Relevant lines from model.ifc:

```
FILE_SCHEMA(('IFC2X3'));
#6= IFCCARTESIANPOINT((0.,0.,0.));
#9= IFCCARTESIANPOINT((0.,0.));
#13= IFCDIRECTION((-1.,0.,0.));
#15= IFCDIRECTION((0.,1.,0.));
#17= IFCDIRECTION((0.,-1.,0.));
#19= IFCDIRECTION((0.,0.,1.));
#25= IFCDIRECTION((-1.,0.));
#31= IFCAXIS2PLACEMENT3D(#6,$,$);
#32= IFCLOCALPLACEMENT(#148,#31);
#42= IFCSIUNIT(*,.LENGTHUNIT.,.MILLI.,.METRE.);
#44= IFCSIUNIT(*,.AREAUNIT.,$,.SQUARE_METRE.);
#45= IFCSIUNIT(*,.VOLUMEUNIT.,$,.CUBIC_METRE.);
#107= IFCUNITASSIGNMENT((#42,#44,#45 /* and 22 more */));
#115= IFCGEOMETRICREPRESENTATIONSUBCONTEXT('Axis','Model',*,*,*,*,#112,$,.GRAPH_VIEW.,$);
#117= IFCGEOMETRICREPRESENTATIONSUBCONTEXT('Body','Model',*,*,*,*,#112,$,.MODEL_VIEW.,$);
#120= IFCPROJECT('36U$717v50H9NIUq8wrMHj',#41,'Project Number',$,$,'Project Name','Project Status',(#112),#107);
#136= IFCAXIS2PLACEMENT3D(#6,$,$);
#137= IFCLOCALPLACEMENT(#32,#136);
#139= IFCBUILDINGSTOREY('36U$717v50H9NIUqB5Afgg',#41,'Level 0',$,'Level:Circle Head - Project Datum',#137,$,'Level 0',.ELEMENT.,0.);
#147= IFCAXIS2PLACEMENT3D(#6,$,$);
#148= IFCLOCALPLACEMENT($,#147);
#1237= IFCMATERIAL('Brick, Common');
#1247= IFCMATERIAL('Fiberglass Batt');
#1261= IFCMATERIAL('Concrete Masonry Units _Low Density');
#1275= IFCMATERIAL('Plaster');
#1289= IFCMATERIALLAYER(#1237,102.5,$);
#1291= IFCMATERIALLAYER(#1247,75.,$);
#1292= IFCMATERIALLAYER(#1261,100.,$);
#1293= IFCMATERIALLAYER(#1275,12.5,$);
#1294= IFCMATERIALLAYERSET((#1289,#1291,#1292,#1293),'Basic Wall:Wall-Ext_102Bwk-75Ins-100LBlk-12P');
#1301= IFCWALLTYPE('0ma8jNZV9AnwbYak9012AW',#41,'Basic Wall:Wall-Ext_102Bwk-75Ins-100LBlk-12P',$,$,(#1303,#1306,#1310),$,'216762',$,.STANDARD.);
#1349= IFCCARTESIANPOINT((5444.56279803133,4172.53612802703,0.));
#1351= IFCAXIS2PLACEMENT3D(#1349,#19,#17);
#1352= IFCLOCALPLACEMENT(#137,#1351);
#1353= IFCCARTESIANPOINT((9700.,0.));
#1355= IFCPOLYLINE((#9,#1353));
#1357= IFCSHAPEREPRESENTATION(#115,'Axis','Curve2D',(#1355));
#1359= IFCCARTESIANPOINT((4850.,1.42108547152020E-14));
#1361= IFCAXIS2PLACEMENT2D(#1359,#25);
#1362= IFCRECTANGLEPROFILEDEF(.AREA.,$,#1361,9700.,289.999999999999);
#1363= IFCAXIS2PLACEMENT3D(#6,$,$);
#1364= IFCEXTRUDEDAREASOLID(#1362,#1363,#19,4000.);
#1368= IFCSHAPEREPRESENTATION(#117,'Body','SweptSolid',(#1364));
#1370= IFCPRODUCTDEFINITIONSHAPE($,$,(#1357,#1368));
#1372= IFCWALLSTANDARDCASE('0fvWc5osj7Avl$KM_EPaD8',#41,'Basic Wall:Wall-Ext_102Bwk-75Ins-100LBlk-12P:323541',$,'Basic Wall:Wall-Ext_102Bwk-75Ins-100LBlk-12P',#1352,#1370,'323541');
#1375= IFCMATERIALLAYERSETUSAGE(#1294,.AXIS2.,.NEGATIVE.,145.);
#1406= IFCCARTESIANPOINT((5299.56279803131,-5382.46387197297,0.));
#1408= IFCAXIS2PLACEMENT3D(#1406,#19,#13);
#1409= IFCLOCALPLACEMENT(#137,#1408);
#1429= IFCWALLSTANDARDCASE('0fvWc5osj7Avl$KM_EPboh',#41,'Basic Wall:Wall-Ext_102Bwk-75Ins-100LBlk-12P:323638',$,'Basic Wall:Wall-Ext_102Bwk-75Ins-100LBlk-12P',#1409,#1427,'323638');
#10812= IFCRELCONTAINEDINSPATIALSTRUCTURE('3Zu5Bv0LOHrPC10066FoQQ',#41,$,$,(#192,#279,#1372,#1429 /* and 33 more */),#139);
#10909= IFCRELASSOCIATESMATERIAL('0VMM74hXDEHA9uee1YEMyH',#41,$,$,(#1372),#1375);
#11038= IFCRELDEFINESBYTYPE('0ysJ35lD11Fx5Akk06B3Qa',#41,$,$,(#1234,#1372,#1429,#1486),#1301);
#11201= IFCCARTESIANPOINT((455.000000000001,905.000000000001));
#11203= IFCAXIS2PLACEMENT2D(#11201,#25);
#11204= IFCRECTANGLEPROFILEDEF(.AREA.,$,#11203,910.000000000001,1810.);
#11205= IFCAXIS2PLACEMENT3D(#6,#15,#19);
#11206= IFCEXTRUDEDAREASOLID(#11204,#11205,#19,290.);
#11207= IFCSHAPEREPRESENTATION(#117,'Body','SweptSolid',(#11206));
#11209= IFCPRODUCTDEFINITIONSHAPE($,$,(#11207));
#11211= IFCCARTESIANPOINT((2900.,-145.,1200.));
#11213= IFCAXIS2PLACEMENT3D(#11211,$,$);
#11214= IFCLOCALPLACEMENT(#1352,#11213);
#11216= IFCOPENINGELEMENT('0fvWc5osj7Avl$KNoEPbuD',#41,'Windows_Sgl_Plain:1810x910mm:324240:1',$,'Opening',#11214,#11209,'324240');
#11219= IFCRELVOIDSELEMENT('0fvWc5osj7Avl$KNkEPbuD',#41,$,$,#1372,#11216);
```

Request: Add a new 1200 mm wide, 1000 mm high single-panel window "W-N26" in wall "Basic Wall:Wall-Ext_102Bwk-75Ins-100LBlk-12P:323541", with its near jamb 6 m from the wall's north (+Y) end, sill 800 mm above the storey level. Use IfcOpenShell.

```python
import numpy as np
import ifcopenshell
import ifcopenshell.api.feature
import ifcopenshell.api.geometry
import ifcopenshell.api.root
import ifcopenshell.api.spatial
import ifcopenshell.api.type
import ifcopenshell.geom
import ifcopenshell.util.element
import ifcopenshell.util.placement
import ifcopenshell.util.representation
import ifcopenshell.util.shape
import ifcopenshell.util.unit

model = ifcopenshell.open("model.ifc")
unit_scale = ifcopenshell.util.unit.calculate_unit_scale(model)
settings = ifcopenshell.geom.settings()


def volume(element):
    """Net volume in cubic metres, openings subtracted."""
    shape = ifcopenshell.geom.create_shape(settings, element)
    return ifcopenshell.util.shape.get_volume(shape.geometry)


wall = model.by_guid("0fvWc5osj7Avl$KM_EPaD8")
storey = ifcopenshell.util.element.get_container(wall, ifc_class="IfcBuildingStorey")
context = ifcopenshell.util.representation.get_context(model, "Model", "Body", "MODEL_VIEW")
before = volume(wall)

width, height, from_end, sill = 1.2, 1, 6, 0.8  # metres

# The wall runs along its own X axis, and the end named is its -X end.
wall_shape = ifcopenshell.geom.create_shape(settings, wall)
x, y, z = ifcopenshell.util.shape.get_vertices(wall_shape.geometry).T
start = x.min() + from_end
face, thickness = float(y.min()), float(y.max() - y.min())
wall_matrix = ifcopenshell.util.placement.get_local_placement(wall.ObjectPlacement)
level = ifcopenshell.util.placement.get_local_placement(storey.ObjectPlacement)[2, 3]


def in_wall(x, y):
    """Placement at x, y metres in the wall's axes, at sill height."""
    matrix = wall_matrix.copy()
    matrix[:, 3] = wall_matrix @ np.array([x / unit_scale, y / unit_scale, 0.0, 1.0])
    matrix[2, 3] = level + sill / unit_scale
    return matrix


# Opening: a box that overshoots both wall faces by 50 mm.
opening = ifcopenshell.api.root.create_entity(model, ifc_class="IfcOpeningElement")
box = ifcopenshell.api.geometry.add_wall_representation(
    model, context=context, length=width, height=height, thickness=thickness + 0.1
)
ifcopenshell.api.geometry.assign_representation(model, product=opening, representation=box)
ifcopenshell.api.geometry.edit_object_placement(model, product=opening, matrix=in_wall(start, face - 0.05), is_si=False)
ifcopenshell.api.feature.add_feature(model, feature=opening, element=wall)

window = ifcopenshell.api.root.create_entity(model, ifc_class="IfcWindow", name="W-N26")
window.OverallWidth, window.OverallHeight = width / unit_scale, height / unit_scale
body = ifcopenshell.api.geometry.add_window_representation(
    model,
    context=context,
    overall_width=window.OverallWidth,
    overall_height=window.OverallHeight,
    partition_type="SINGLE_PANEL",
)
ifcopenshell.api.geometry.assign_representation(model, product=window, representation=body)
ifcopenshell.api.spatial.assign_container(model, products=[window], relating_structure=storey)
fills = ifcopenshell.api.feature.add_filling(model, opening=opening, element=window)
fills.OwnerHistory = window.OwnerHistory  # required in IFC2X3

# IFC2X3 keeps the operation on the window style.
style = ifcopenshell.api.root.create_entity(model, ifc_class="IfcWindowStyle", name="W-N26")
style.OperationType, style.ConstructionType = "SINGLE_PANEL", "NOTDEFINED"
style.ParameterTakesPrecedence = style.Sizeable = False
ifcopenshell.api.type.assign_type(model, related_objects=[window], relating_type=style)

# Centre the window in the wall's thickness.
ifcopenshell.api.geometry.edit_object_placement(model, product=window, matrix=in_wall(start, face), is_si=False)
window_shape = ifcopenshell.geom.create_shape(settings, window)
depth = ifcopenshell.util.shape.get_vertices(window_shape.geometry)[:, 1]
offset = face + thickness / 2 - (depth.min() + depth.max()) / 2
ifcopenshell.api.geometry.edit_object_placement(model, product=window, matrix=in_wall(start, offset), is_si=False)

after = volume(wall)

print(f"wall volume {before:.3f} -> {after:.3f} m3")

model.write("model_edited.ifc")
```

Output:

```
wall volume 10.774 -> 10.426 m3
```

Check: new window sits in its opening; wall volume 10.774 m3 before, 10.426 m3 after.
